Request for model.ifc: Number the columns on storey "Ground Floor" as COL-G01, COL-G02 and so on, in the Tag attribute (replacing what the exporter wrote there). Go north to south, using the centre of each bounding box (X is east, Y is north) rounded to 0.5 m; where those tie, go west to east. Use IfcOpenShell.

First a look at what the model holds.

```python
import ifcopenshell
import ifcopenshell.util.element
import ifcopenshell.util.placement

model = ifcopenshell.open("model.ifc")
print(model.schema)
storey = next(s for s in model.by_type("IfcBuildingStorey") if s.Name == "Ground Floor")
columns = [e for e in ifcopenshell.util.element.get_decomposition(storey) if e.is_a("IfcColumn")]
for e in sorted(columns, key=lambda e: e.id()):
    origin = ifcopenshell.util.placement.get_local_placement(e.ObjectPlacement)[:3, 3]
    print(e.id(), e.Tag, e.Name, origin.round(2) + 0.0, sep=" | ")
```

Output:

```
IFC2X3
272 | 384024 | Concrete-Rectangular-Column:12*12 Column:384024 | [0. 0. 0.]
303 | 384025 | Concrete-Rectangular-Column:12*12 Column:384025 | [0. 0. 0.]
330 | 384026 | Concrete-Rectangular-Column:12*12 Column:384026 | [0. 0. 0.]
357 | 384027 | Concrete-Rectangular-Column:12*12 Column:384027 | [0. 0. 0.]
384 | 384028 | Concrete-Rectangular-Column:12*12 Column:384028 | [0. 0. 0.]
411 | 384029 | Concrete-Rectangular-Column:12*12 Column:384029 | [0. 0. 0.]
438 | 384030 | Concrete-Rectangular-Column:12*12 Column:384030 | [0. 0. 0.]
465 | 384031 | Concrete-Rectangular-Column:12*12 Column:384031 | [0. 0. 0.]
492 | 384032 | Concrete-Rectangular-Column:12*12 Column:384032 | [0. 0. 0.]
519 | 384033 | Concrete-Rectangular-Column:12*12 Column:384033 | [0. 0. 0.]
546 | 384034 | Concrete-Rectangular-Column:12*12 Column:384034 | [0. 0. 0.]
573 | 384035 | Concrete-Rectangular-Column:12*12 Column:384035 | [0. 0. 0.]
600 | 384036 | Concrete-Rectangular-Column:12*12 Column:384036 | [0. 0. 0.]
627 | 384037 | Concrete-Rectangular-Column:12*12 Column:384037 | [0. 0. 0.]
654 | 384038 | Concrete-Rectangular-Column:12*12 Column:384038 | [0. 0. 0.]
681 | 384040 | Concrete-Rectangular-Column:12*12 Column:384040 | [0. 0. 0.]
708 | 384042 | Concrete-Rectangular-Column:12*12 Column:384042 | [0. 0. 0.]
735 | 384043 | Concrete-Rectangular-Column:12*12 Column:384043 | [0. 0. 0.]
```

```python
import ifcopenshell
import ifcopenshell.geom
import ifcopenshell.util.element
import ifcopenshell.util.shape

model = ifcopenshell.open("model.ifc")
settings = ifcopenshell.geom.settings()
settings.set("use-world-coords", True)


def centre(element):
    shape = ifcopenshell.geom.create_shape(settings, element)
    return ifcopenshell.util.shape.get_bbox_centroid(shape.geometry)


storey = next(s for s in model.by_type("IfcBuildingStorey") if s.Name == "Ground Floor")
columns = [e for e in ifcopenshell.util.element.get_decomposition(storey) if e.is_a("IfcColumn")]

# Insertion points can sit at a corner or the storey origin, so sort by the geometry (in metres).
centres = {e: centre(e) for e in columns}
columns.sort(key=lambda e: (-round(centres[e][1] / 0.5), centres[e][0]))

for i, e in enumerate(columns, start=1):
    number = f"COL-G{i:02d}"
    e.Tag = number
    print(e.id(), number)

model.write("model_updated.ifc")
```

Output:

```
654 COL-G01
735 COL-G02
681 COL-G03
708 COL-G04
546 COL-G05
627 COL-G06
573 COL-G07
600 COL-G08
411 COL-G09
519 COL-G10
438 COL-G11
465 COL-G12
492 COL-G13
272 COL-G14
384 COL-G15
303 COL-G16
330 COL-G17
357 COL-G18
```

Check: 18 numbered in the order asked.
